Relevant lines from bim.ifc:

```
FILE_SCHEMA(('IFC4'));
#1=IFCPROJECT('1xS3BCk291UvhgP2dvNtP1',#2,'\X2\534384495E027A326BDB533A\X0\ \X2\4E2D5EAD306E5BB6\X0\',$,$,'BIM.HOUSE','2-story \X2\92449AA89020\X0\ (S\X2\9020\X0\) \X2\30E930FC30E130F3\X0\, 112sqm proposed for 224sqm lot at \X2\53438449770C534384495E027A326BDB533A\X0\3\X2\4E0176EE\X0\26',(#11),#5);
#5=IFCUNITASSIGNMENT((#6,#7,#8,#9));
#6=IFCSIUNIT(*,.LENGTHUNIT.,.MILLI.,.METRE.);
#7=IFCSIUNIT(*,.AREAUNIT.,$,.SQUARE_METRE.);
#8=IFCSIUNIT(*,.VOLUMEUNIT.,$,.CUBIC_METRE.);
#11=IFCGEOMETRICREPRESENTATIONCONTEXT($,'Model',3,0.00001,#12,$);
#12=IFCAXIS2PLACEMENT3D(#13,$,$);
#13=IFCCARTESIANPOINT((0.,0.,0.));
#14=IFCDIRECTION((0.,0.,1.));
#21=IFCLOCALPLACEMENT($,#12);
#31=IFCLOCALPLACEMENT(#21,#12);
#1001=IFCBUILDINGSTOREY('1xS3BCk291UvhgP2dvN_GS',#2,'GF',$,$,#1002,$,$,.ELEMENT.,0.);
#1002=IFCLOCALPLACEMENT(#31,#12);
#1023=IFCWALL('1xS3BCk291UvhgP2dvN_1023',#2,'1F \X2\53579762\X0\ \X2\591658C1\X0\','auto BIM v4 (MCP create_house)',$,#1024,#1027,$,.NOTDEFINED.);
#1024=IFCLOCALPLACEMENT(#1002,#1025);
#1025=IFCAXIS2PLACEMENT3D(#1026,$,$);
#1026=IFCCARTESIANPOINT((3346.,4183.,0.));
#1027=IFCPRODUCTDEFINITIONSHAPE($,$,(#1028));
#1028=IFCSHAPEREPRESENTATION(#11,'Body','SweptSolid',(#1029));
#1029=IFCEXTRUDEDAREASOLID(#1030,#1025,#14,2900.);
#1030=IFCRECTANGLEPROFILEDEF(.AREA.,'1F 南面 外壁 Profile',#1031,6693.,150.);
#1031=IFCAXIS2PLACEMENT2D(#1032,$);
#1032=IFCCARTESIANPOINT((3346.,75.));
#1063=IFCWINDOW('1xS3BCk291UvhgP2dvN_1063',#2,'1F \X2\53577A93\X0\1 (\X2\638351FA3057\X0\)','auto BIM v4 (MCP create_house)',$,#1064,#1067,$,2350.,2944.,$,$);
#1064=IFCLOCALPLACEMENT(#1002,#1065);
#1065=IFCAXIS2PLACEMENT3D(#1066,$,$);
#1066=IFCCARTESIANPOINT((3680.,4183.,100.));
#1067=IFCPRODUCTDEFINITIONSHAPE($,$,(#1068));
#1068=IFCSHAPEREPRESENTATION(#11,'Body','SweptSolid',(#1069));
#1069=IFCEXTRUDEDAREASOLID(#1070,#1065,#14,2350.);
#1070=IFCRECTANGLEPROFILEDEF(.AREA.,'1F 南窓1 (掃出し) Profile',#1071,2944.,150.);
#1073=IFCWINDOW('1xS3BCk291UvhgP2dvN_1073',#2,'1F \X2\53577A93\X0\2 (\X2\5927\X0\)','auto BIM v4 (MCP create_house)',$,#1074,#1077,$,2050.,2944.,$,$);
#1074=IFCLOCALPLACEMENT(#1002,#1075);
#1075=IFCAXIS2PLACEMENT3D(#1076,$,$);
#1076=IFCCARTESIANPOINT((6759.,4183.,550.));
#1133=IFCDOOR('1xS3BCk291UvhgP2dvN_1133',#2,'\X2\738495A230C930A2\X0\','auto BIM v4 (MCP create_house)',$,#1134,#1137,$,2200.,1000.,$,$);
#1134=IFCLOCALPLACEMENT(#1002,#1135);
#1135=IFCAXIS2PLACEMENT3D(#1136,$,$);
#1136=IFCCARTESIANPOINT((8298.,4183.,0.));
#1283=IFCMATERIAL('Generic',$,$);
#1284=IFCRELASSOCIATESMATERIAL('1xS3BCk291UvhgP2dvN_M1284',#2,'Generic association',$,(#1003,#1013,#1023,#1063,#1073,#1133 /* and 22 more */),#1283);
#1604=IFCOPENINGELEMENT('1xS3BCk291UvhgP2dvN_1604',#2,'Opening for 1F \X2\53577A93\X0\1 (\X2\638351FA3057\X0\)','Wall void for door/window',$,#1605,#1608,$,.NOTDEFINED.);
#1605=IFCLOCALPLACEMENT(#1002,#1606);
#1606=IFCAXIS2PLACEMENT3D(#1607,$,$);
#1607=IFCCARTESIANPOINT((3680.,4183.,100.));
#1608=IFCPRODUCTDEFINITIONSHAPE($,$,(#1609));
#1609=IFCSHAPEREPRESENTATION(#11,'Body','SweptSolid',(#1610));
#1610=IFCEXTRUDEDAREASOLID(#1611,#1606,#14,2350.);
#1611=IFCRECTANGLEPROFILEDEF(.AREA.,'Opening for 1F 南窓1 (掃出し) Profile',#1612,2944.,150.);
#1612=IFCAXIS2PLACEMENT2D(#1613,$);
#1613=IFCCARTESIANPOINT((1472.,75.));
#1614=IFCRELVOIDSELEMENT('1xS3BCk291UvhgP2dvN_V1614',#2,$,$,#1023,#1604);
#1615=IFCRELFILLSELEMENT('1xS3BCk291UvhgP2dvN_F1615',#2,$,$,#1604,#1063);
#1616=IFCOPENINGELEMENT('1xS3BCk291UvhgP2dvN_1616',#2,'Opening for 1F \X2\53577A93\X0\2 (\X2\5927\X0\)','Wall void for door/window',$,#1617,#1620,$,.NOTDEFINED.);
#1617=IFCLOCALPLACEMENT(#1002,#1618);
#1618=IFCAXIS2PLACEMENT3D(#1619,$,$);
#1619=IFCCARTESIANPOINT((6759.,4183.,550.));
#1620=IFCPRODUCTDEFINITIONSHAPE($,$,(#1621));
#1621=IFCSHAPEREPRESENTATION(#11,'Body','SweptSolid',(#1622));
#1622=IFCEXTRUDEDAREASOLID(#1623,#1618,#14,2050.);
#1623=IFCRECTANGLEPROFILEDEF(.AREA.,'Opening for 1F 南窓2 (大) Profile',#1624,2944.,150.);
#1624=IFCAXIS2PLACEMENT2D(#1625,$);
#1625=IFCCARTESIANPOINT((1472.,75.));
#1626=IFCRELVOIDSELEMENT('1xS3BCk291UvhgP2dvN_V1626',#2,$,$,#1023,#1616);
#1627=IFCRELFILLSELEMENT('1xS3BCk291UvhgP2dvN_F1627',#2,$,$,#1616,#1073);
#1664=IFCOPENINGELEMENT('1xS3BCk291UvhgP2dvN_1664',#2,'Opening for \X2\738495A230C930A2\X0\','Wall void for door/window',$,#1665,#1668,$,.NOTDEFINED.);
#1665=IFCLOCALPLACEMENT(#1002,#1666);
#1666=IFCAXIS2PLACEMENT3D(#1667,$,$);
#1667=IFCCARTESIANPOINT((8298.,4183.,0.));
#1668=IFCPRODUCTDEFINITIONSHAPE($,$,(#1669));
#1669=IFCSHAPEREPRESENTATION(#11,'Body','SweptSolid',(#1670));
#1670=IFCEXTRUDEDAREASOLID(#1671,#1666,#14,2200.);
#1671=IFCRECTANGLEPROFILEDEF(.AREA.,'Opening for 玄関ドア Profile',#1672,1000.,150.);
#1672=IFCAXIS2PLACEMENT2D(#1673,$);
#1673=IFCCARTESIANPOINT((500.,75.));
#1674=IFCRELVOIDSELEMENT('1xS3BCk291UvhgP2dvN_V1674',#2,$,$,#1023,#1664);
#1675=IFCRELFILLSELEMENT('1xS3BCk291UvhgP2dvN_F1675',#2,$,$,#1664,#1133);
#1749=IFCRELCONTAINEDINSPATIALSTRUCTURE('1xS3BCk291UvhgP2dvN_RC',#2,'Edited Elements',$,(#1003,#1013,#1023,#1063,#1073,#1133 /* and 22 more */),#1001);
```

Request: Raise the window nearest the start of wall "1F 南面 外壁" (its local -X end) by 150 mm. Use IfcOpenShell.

```python
import numpy as np
import ifcopenshell
import ifcopenshell.api.geometry
import ifcopenshell.util.placement
import ifcopenshell.util.unit

model = ifcopenshell.open("bim.ifc")
unit_scale = ifcopenshell.util.unit.calculate_unit_scale(model)

window = model.by_guid("1xS3BCk291UvhgP2dvN_1063")
opening = window.FillsVoids[0].RelatingOpeningElement
dz = 0.15 / unit_scale

shift = np.array([0.0, 0.0, dz])
# The window is not placed relative to its opening, so move both.
for product in (opening, window):
    matrix = ifcopenshell.util.placement.get_local_placement(product.ObjectPlacement)
    matrix[:3, 3] += shift
    ifcopenshell.api.geometry.edit_object_placement(model, product=product, matrix=matrix, is_si=False)

print(f"moved by {dz * unit_scale:+.3f} m")

model.write("bim_updated.ifc")
```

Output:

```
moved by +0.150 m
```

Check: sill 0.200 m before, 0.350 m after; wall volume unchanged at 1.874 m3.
